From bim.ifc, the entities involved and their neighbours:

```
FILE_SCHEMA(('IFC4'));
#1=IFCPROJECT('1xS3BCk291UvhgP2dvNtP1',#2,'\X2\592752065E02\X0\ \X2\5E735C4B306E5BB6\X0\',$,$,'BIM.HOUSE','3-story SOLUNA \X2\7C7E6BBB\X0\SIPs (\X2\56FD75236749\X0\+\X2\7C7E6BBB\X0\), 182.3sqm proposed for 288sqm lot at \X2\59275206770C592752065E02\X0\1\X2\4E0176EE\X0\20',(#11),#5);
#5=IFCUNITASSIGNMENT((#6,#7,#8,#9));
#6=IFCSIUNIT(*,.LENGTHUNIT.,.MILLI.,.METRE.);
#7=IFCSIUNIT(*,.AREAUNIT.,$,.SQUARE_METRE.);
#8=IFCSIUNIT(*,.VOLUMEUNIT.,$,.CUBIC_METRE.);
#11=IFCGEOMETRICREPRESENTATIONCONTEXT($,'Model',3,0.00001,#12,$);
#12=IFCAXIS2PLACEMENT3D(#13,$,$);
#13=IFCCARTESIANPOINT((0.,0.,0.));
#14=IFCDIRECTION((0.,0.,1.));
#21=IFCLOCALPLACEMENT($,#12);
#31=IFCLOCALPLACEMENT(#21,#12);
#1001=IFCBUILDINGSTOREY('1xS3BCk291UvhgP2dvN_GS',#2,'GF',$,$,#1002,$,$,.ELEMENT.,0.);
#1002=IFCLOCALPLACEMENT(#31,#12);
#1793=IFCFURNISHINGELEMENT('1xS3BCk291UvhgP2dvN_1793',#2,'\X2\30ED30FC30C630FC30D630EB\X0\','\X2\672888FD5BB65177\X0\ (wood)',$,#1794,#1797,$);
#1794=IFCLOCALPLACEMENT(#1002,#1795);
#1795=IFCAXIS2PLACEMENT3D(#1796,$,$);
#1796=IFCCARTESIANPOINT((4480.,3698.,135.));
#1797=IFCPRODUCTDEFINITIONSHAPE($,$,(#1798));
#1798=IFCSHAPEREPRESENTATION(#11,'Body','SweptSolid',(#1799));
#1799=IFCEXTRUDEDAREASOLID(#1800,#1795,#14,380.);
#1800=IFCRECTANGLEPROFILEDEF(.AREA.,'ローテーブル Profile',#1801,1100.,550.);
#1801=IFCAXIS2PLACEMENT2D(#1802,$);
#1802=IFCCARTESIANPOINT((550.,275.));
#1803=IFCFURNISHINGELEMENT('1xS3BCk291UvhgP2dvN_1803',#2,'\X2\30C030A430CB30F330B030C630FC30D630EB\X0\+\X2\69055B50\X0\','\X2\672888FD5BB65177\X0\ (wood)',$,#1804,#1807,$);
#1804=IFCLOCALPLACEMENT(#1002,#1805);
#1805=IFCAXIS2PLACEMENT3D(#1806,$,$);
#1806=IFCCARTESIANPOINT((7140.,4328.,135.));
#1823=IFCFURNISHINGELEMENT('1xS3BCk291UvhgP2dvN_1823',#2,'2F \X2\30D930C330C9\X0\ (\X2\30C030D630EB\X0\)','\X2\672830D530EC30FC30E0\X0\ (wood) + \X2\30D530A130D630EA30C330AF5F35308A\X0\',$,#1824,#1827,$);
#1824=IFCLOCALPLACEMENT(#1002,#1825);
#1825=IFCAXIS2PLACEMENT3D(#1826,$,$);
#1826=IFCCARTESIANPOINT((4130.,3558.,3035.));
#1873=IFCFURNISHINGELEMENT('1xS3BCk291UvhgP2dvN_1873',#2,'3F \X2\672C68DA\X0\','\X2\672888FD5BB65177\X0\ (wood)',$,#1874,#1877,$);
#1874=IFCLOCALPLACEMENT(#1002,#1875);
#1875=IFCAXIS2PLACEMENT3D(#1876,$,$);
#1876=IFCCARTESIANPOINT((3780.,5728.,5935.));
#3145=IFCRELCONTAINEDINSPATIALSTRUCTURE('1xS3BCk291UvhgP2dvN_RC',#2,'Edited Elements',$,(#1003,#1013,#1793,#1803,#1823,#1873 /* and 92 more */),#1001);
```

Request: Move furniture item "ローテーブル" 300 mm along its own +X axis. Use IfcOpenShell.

```python
import ifcopenshell
import ifcopenshell.api.geometry
import ifcopenshell.util.placement
import ifcopenshell.util.unit

model = ifcopenshell.open("bim.ifc")
unit_scale = ifcopenshell.util.unit.calculate_unit_scale(model)

item = model.by_guid("1xS3BCk291UvhgP2dvN_1793")
matrix = ifcopenshell.util.placement.get_local_placement(item.ObjectPlacement)
matrix[:3, 3] += matrix[:3, 0] * 0.3 / unit_scale
ifcopenshell.api.geometry.edit_object_placement(model, product=item, matrix=matrix, is_si=False)

print(ifcopenshell.util.placement.get_local_placement(item.ObjectPlacement).round(3) + 0.0)

model.write("bim_edited.ifc")
```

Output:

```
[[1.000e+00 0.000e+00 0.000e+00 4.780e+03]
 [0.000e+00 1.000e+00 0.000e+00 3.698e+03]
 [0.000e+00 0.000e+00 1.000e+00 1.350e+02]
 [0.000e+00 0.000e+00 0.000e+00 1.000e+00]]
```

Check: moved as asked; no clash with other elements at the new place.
